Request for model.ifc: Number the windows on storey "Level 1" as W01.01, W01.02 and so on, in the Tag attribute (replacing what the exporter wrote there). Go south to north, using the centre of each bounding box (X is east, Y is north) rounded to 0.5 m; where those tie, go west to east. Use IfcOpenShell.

First a look at what the model holds.

```python
import ifcopenshell
import ifcopenshell.util.element
import ifcopenshell.util.placement

model = ifcopenshell.open("model.ifc")
print(model.schema)
storey = next(s for s in model.by_type("IfcBuildingStorey") if s.Name == "Level 1")
windows = [e for e in ifcopenshell.util.element.get_decomposition(storey) if e.is_a("IfcWindow")]
for e in sorted(windows, key=lambda e: e.id()):
    origin = ifcopenshell.util.placement.get_local_placement(e.ObjectPlacement)[:3, 3]
    print(e.id(), e.Tag, e.Name, origin.round(2) + 0.0, sep=" | ")
```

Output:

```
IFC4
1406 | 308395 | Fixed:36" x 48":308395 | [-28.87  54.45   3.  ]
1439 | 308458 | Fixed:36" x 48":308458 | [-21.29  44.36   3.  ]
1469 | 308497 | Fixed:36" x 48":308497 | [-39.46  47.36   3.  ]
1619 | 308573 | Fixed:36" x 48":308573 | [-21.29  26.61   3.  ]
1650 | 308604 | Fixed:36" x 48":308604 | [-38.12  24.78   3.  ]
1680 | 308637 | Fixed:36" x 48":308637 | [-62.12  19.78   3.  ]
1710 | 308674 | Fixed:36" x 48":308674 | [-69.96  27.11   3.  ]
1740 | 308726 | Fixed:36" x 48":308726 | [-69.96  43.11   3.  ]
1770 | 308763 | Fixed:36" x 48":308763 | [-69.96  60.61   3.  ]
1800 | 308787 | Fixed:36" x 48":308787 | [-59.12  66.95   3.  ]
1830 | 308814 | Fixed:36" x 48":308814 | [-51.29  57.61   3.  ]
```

```python
import ifcopenshell
import ifcopenshell.geom
import ifcopenshell.util.element
import ifcopenshell.util.shape

model = ifcopenshell.open("model.ifc")
settings = ifcopenshell.geom.settings()
settings.set("use-world-coords", True)


def centre(element):
    shape = ifcopenshell.geom.create_shape(settings, element)
    return ifcopenshell.util.shape.get_bbox_centroid(shape.geometry)


storey = next(s for s in model.by_type("IfcBuildingStorey") if s.Name == "Level 1")
windows = [e for e in ifcopenshell.util.element.get_decomposition(storey) if e.is_a("IfcWindow")]

# Insertion points can sit at a corner or the storey origin, so sort by the geometry (in metres).
centres = {e: centre(e) for e in windows}
windows.sort(key=lambda e: (round(centres[e][1] / 0.5), centres[e][0]))

for i, e in enumerate(windows, start=1):
    number = f"W01.{i:02d}"
    e.Tag = number
    print(e.id(), number)

model.write("model_edited.ifc")
```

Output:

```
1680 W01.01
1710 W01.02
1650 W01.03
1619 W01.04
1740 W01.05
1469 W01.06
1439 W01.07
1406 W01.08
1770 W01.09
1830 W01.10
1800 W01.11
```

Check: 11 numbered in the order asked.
